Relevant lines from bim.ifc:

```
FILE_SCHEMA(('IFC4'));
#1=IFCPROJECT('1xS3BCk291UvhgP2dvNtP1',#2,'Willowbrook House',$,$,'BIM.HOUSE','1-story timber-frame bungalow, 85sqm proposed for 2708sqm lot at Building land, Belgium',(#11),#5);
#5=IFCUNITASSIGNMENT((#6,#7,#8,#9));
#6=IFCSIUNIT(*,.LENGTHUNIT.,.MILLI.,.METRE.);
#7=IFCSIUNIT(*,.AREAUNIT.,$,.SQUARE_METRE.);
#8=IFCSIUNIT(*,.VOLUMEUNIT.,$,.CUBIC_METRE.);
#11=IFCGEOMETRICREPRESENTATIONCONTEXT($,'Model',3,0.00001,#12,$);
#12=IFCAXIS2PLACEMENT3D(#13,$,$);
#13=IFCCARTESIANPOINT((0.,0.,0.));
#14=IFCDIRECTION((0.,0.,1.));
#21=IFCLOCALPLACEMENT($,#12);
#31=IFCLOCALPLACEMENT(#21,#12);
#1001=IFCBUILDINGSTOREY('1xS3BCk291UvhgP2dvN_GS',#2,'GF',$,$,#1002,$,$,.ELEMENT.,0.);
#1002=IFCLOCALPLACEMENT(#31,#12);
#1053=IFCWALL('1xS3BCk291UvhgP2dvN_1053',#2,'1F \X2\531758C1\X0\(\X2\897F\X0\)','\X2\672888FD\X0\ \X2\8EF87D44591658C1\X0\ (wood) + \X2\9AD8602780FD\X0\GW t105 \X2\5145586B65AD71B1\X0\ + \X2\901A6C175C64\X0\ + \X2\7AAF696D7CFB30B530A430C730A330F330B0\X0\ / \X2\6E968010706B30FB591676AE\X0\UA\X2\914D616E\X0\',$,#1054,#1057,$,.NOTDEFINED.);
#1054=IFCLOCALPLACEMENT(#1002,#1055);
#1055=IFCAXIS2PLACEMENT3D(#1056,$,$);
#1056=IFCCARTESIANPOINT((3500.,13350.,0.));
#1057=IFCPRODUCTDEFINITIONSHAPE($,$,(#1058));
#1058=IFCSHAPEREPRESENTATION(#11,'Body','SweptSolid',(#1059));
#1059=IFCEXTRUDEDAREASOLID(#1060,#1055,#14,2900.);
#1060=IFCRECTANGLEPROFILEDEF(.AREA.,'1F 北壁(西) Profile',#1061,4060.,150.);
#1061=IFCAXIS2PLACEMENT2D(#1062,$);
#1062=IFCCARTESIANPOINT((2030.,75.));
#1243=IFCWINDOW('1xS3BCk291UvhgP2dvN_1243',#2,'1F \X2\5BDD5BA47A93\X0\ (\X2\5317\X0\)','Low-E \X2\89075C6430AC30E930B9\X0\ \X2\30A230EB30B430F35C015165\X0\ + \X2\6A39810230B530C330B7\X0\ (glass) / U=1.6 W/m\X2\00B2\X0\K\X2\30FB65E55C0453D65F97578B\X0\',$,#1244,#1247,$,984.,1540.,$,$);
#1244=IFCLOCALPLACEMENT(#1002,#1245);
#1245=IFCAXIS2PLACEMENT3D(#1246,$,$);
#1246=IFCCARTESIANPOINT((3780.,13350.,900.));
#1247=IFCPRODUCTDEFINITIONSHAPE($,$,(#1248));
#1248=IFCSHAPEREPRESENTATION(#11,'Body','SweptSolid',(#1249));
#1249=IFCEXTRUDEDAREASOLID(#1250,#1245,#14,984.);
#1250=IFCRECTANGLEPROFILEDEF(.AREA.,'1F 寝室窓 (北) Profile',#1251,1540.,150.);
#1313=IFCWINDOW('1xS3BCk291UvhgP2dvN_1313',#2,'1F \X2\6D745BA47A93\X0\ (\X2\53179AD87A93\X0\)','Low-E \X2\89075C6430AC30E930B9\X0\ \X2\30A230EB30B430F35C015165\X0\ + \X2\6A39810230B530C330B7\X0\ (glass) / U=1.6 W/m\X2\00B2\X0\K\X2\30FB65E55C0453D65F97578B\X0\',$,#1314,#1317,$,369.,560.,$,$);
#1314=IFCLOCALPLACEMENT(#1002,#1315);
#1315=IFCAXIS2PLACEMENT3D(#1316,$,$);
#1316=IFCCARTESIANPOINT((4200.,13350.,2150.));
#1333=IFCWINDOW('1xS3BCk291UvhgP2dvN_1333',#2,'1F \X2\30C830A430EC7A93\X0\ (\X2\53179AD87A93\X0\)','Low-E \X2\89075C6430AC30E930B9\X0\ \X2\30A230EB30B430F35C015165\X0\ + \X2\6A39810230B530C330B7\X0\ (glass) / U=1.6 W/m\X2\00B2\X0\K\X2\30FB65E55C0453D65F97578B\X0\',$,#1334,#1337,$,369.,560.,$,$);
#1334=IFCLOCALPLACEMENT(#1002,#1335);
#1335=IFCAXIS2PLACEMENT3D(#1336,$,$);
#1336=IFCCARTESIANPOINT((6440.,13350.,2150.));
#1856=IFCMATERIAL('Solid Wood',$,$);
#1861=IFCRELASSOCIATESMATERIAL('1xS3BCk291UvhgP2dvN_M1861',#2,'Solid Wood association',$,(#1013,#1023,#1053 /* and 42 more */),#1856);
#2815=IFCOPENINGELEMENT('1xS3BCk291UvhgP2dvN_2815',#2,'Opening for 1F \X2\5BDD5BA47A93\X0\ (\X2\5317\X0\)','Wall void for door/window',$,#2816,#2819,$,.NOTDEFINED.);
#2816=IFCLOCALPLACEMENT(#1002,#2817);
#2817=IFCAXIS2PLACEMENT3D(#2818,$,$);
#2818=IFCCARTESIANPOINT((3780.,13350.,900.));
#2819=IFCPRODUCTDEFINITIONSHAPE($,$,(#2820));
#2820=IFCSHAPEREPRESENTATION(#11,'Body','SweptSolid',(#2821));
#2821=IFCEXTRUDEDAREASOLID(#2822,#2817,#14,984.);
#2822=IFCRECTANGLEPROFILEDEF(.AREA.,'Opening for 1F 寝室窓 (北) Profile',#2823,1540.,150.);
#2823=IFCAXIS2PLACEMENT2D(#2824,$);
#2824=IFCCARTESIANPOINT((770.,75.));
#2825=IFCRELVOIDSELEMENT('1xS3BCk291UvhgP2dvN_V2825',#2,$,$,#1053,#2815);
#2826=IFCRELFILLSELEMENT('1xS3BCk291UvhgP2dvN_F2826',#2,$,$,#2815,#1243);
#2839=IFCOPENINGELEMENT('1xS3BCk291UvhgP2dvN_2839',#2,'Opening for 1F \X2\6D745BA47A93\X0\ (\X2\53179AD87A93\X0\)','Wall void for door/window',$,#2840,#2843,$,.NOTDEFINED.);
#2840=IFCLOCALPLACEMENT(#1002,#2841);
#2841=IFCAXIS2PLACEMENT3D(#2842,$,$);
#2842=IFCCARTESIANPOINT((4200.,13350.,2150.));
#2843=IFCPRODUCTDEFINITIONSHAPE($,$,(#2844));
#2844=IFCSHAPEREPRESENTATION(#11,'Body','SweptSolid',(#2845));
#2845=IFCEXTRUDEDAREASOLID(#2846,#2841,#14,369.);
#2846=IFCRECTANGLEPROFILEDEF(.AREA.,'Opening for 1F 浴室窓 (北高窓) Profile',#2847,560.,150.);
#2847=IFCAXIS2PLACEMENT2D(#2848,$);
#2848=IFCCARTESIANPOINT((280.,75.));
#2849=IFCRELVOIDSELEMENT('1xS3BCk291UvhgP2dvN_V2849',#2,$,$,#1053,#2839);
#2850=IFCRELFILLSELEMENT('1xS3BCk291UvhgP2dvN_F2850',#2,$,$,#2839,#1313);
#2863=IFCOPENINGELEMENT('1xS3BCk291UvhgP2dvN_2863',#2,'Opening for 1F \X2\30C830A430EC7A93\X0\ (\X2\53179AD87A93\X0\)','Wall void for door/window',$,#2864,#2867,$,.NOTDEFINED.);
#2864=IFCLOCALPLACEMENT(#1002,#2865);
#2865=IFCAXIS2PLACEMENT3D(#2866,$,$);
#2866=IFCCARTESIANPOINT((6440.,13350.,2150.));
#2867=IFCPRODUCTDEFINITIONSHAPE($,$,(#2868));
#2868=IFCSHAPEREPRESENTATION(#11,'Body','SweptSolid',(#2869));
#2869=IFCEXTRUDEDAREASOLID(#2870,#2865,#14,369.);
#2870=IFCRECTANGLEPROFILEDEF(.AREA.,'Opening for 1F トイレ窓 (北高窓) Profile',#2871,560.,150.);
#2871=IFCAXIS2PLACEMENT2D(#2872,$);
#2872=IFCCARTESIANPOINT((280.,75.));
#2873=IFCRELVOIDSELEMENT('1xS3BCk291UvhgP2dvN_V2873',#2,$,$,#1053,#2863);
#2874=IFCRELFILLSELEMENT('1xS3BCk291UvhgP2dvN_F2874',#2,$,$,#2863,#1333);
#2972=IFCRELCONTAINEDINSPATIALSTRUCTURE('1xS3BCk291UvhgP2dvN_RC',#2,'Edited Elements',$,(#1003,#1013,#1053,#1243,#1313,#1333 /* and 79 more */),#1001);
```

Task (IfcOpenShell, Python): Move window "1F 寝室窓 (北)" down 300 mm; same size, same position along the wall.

```python
import numpy as np
import ifcopenshell
import ifcopenshell.api.geometry
import ifcopenshell.util.placement
import ifcopenshell.util.unit

model = ifcopenshell.open("bim.ifc")
unit_scale = ifcopenshell.util.unit.calculate_unit_scale(model)

window = model.by_guid("1xS3BCk291UvhgP2dvN_1243")
opening = window.FillsVoids[0].RelatingOpeningElement
dz = -300.0

shift = np.array([0.0, 0.0, dz])
# The window is not placed relative to its opening, so move both.
for product in (opening, window):
    matrix = ifcopenshell.util.placement.get_local_placement(product.ObjectPlacement)
    matrix[:3, 3] += shift
    ifcopenshell.api.geometry.edit_object_placement(model, product=product, matrix=matrix, is_si=False)

print(f"moved by {dz * unit_scale:+.3f} m")

model.write("bim_rev.ifc")
```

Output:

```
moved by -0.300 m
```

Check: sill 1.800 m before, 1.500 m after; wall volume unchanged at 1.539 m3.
